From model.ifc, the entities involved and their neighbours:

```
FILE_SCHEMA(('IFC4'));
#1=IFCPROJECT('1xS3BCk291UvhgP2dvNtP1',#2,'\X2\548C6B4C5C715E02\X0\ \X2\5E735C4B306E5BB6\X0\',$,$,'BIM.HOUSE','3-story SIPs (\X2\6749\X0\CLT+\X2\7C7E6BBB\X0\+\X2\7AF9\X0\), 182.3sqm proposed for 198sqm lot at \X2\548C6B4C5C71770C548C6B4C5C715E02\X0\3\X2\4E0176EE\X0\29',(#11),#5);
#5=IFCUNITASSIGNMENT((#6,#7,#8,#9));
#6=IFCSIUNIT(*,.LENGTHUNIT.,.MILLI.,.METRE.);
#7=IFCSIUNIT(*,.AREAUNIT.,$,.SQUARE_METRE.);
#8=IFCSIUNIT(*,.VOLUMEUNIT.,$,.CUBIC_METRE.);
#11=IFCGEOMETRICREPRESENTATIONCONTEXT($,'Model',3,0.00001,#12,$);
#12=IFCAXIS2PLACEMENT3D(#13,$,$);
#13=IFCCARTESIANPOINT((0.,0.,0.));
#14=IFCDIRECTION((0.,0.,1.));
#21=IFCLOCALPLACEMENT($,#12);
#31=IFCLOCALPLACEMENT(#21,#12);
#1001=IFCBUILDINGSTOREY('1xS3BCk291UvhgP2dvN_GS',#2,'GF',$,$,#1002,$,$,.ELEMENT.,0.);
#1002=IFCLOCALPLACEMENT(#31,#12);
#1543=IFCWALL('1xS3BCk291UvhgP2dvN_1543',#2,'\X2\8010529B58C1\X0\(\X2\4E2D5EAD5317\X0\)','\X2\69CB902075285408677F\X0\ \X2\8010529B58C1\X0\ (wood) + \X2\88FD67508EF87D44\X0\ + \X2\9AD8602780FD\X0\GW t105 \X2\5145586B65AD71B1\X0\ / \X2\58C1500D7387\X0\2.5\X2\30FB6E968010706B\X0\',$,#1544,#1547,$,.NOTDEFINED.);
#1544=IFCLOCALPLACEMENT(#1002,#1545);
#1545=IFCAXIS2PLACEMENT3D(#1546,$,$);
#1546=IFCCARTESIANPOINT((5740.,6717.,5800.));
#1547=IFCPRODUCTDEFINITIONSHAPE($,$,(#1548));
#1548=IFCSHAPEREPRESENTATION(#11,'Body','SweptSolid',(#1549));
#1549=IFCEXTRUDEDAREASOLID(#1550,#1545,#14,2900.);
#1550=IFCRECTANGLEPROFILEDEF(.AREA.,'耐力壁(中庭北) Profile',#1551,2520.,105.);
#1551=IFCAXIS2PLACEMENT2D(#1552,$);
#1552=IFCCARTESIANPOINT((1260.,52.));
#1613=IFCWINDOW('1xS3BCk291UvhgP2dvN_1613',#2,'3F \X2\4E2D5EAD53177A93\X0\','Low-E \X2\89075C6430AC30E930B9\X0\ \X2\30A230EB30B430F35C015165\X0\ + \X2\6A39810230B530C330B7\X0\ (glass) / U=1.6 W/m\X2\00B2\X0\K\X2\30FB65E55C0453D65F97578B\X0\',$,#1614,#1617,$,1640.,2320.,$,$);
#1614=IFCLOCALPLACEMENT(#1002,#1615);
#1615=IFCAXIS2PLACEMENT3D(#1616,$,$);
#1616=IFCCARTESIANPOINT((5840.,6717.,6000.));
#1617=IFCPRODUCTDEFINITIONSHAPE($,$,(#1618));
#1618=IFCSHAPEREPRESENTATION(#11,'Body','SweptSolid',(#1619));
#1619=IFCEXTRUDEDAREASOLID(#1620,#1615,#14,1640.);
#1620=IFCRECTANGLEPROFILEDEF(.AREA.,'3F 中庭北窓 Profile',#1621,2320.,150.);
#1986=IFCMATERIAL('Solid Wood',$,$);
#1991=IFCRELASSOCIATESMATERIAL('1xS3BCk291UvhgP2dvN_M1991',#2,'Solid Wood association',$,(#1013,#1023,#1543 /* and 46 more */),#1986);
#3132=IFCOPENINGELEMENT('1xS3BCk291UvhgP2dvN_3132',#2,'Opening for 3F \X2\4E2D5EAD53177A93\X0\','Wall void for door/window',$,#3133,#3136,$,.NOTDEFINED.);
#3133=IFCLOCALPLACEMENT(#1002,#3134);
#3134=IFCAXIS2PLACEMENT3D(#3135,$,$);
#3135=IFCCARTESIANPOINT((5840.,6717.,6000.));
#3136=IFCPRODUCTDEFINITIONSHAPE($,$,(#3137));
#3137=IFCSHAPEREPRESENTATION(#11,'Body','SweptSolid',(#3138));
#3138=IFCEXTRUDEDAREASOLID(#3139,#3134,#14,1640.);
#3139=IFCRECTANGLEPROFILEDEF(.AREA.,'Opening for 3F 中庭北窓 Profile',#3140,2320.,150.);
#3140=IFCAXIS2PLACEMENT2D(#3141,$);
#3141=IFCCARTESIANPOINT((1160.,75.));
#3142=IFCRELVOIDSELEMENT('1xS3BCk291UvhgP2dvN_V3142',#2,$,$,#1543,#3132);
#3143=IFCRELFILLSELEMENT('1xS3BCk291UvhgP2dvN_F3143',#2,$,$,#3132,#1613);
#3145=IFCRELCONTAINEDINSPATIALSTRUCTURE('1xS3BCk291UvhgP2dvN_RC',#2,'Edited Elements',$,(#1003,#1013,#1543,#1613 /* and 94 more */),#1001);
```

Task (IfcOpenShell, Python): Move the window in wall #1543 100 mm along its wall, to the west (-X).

```python
import ifcopenshell
import ifcopenshell.api.geometry
import ifcopenshell.util.placement
import ifcopenshell.util.unit

model = ifcopenshell.open("model.ifc")
unit_scale = ifcopenshell.util.unit.calculate_unit_scale(model)

window = model.by_guid("1xS3BCk291UvhgP2dvN_1613")
opening = window.FillsVoids[0].RelatingOpeningElement
wall = opening.VoidsElements[0].RelatingBuildingElement

wall_matrix = ifcopenshell.util.placement.get_local_placement(wall.ObjectPlacement)
shift = wall_matrix[:3, 0] * -0.1 / unit_scale
before = ifcopenshell.util.placement.get_local_placement(window.ObjectPlacement)[:3, 3].copy()

# The window is not placed relative to its opening, so move both.
for product in (opening, window):
    matrix = ifcopenshell.util.placement.get_local_placement(product.ObjectPlacement)
    matrix[:3, 3] += shift
    ifcopenshell.api.geometry.edit_object_placement(model, product=product, matrix=matrix, is_si=False)

after = ifcopenshell.util.placement.get_local_placement(window.ObjectPlacement)[:3, 3]
print("window moved by", (after - before).round(3) + 0.0)

model.write("model_rev.ifc")
```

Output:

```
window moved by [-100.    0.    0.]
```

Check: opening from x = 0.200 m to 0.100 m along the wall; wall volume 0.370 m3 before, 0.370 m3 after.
